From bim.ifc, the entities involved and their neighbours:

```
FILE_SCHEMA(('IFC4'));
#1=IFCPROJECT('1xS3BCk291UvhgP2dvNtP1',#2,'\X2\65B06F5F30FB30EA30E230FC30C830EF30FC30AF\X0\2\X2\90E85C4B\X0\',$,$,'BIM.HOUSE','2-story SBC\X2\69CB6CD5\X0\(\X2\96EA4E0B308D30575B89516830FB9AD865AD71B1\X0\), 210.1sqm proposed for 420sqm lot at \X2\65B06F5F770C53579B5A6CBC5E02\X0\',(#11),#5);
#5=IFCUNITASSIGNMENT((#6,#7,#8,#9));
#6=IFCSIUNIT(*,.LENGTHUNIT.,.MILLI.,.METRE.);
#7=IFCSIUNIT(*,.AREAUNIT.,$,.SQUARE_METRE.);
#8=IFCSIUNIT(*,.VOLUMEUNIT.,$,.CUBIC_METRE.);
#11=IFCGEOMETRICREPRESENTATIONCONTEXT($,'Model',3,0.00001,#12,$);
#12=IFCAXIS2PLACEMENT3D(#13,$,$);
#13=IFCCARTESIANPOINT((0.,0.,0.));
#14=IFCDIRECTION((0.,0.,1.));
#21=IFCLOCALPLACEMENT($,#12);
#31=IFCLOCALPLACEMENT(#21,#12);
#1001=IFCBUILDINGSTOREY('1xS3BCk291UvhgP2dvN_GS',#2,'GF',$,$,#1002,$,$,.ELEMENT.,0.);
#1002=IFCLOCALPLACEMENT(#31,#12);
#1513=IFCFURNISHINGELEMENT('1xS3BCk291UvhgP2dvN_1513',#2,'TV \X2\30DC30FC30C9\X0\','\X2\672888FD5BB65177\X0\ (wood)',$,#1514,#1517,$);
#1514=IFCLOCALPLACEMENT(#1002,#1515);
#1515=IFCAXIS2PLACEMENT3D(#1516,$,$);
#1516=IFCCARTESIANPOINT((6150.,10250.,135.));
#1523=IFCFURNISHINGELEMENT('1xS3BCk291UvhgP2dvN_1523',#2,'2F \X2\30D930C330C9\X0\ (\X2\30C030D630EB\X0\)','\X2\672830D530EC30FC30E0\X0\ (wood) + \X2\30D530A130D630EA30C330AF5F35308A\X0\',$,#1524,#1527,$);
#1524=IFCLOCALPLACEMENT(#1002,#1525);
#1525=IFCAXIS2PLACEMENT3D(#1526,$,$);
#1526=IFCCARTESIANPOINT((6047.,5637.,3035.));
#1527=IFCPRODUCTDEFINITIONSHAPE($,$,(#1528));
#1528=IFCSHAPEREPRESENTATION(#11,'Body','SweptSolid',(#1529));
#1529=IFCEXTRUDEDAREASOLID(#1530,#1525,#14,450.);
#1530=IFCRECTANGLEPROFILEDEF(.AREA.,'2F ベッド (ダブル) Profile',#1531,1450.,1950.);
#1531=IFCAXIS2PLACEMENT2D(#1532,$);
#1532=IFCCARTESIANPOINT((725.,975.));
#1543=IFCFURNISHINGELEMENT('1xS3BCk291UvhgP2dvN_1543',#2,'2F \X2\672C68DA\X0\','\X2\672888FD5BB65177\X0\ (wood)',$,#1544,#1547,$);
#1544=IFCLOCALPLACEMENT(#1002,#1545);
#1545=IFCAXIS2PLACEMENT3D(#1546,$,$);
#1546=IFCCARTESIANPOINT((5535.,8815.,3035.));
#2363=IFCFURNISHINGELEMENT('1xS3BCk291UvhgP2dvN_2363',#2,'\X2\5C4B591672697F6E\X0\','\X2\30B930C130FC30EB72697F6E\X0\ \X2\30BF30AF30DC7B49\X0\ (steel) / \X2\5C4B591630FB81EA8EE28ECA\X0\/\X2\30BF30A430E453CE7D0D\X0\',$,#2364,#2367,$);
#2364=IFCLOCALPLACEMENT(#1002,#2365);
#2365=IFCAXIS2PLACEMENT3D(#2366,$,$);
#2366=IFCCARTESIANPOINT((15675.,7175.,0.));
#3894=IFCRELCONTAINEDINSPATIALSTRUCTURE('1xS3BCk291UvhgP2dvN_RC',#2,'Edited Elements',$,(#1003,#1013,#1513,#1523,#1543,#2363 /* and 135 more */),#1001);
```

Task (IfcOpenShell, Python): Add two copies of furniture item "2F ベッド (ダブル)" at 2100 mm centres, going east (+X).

```python
import numpy as np
import ifcopenshell
import ifcopenshell.api.geometry
import ifcopenshell.api.root
import ifcopenshell.util.element
import ifcopenshell.util.placement
import ifcopenshell.util.unit

model = ifcopenshell.open("bim.ifc")
unit_scale = ifcopenshell.util.unit.calculate_unit_scale(model)


def reuse_history(source, copy):
    """copy_class also copies each property set's owner history, people and application; keep the originals."""
    for rel in copy.IsDefinedBy:
        if rel.is_a("IfcRelDefinesByProperties") and (history := rel.RelatingPropertyDefinition.OwnerHistory):
            rel.RelatingPropertyDefinition.OwnerHistory = source.OwnerHistory
            ifcopenshell.util.element.remove_deep2(model, history)


source = model.by_id(1523)
base = ifcopenshell.util.placement.get_local_placement(source.ObjectPlacement)
step = np.array([1.0, 0.0, 0.0]) * 2.1 / unit_scale

for i in range(1, 3):
    copy = ifcopenshell.api.root.copy_class(model, product=source)
    copy.Representation = ifcopenshell.util.element.copy_deep(
        model, source.Representation, exclude=["IfcGeometricRepresentationContext", "IfcRepresentationMap"]
    )
    reuse_history(source, copy)
    matrix = base.copy()
    matrix[:3, 3] += i * step
    print("added at", matrix[:3, 3].round(3) + 0.0)
    ifcopenshell.api.geometry.edit_object_placement(model, product=copy, matrix=matrix, is_si=False)

model.write("bim_rev.ifc")
```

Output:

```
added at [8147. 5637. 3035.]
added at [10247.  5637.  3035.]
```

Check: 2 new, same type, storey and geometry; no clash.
